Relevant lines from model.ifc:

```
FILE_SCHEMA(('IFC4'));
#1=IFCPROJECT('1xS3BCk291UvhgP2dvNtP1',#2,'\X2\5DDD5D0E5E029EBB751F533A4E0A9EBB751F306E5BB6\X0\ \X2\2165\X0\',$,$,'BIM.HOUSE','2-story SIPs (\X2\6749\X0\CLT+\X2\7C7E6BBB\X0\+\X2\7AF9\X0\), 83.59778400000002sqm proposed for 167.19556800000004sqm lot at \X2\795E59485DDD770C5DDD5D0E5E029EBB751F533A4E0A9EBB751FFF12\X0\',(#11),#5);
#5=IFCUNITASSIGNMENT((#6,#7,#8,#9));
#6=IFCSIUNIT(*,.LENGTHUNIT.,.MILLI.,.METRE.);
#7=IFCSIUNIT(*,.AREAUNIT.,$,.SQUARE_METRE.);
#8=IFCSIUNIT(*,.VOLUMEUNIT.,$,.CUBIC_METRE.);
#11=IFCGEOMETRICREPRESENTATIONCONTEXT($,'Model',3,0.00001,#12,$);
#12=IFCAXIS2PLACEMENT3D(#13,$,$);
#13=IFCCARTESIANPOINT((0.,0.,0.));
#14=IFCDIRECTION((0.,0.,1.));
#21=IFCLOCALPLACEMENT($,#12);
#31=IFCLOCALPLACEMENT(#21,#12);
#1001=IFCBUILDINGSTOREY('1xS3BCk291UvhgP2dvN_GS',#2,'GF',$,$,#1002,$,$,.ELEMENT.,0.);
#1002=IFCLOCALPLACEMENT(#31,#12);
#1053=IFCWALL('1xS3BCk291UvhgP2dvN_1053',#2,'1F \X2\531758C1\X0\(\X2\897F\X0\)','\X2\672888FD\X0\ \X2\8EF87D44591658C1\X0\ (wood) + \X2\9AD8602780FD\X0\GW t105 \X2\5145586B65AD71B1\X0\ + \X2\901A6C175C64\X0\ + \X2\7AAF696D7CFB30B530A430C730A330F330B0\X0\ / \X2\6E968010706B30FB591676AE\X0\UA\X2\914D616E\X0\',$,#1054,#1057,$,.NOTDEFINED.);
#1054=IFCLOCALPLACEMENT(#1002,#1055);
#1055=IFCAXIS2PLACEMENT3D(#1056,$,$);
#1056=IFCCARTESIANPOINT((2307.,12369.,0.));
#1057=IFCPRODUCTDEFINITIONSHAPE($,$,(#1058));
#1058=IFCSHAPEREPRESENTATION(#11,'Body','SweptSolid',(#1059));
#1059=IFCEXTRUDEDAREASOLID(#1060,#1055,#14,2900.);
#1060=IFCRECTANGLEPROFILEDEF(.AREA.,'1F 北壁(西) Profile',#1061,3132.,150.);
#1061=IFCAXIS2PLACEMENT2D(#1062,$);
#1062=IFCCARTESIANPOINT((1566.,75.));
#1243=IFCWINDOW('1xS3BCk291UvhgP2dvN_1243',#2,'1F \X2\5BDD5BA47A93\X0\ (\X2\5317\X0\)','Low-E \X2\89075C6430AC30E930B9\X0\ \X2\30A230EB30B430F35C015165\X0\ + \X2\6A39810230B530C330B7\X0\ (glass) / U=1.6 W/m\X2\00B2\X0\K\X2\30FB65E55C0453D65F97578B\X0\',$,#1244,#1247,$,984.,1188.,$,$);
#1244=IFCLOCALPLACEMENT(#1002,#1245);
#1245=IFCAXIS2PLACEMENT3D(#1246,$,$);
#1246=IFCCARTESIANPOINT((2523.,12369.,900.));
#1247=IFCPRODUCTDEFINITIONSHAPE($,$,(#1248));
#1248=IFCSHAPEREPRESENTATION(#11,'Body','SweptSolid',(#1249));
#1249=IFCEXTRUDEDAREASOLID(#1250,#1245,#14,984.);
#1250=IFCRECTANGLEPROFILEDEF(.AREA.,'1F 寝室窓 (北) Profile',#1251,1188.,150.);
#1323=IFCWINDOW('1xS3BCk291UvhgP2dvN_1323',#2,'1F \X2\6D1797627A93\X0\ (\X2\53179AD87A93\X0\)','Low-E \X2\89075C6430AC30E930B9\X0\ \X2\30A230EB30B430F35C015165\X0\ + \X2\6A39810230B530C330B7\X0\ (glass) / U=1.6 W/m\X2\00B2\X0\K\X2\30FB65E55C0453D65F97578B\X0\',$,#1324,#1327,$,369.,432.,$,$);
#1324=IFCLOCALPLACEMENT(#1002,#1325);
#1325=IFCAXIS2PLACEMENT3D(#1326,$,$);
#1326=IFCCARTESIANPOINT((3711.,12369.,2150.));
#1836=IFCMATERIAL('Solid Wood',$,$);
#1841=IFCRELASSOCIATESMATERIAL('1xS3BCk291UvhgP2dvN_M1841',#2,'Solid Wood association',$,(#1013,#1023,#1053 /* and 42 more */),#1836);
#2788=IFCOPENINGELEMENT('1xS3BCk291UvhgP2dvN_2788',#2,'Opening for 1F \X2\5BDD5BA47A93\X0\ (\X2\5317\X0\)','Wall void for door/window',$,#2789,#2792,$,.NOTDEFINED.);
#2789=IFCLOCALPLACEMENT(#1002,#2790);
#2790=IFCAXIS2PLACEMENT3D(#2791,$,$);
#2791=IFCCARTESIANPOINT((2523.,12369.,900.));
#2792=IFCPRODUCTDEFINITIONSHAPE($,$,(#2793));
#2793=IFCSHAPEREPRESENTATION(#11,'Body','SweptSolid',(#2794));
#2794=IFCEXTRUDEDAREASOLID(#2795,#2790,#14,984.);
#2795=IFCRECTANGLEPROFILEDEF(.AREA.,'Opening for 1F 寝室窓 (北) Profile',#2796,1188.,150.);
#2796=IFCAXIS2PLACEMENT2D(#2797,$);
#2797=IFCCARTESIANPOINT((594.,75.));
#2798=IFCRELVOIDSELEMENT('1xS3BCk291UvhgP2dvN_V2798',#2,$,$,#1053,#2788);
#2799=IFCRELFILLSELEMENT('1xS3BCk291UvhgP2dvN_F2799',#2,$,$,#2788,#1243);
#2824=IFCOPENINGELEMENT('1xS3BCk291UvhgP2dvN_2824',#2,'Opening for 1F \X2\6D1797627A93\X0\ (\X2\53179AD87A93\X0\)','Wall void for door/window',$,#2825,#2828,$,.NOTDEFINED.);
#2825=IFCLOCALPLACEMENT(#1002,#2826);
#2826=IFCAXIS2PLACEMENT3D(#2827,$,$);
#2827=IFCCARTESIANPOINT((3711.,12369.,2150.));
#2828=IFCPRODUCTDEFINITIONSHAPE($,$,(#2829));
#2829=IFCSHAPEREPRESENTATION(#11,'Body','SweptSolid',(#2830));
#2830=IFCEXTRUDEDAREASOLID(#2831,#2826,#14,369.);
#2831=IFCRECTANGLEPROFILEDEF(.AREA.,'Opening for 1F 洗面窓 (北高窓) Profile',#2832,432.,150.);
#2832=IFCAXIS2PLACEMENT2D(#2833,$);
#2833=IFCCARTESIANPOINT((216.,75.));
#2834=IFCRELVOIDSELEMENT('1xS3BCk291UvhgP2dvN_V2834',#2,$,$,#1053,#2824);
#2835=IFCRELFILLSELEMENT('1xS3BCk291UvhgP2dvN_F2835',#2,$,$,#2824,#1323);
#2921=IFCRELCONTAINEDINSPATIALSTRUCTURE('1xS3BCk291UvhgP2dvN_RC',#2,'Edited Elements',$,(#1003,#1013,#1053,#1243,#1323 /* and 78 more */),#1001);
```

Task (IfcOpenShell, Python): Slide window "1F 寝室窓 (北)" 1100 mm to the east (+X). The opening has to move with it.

```python
import ifcopenshell
import ifcopenshell.api.geometry
import ifcopenshell.util.placement
import ifcopenshell.util.unit

model = ifcopenshell.open("model.ifc")
unit_scale = ifcopenshell.util.unit.calculate_unit_scale(model)

window = model.by_guid("1xS3BCk291UvhgP2dvN_1243")
opening = window.FillsVoids[0].RelatingOpeningElement
wall = opening.VoidsElements[0].RelatingBuildingElement

wall_matrix = ifcopenshell.util.placement.get_local_placement(wall.ObjectPlacement)
shift = wall_matrix[:3, 0] * 1.1 / unit_scale
before = ifcopenshell.util.placement.get_local_placement(window.ObjectPlacement)[:3, 3].copy()

# The window is not placed relative to its opening, so move both.
for product in (opening, window):
    matrix = ifcopenshell.util.placement.get_local_placement(product.ObjectPlacement)
    matrix[:3, 3] += shift
    ifcopenshell.api.geometry.edit_object_placement(model, product=product, matrix=matrix, is_si=False)

after = ifcopenshell.util.placement.get_local_placement(window.ObjectPlacement)[:3, 3]
print("window moved by", (after - before).round(3) + 0.0)

model.write("model_edited.ifc")
```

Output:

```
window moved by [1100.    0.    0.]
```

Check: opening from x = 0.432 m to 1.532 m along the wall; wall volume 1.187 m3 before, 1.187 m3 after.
